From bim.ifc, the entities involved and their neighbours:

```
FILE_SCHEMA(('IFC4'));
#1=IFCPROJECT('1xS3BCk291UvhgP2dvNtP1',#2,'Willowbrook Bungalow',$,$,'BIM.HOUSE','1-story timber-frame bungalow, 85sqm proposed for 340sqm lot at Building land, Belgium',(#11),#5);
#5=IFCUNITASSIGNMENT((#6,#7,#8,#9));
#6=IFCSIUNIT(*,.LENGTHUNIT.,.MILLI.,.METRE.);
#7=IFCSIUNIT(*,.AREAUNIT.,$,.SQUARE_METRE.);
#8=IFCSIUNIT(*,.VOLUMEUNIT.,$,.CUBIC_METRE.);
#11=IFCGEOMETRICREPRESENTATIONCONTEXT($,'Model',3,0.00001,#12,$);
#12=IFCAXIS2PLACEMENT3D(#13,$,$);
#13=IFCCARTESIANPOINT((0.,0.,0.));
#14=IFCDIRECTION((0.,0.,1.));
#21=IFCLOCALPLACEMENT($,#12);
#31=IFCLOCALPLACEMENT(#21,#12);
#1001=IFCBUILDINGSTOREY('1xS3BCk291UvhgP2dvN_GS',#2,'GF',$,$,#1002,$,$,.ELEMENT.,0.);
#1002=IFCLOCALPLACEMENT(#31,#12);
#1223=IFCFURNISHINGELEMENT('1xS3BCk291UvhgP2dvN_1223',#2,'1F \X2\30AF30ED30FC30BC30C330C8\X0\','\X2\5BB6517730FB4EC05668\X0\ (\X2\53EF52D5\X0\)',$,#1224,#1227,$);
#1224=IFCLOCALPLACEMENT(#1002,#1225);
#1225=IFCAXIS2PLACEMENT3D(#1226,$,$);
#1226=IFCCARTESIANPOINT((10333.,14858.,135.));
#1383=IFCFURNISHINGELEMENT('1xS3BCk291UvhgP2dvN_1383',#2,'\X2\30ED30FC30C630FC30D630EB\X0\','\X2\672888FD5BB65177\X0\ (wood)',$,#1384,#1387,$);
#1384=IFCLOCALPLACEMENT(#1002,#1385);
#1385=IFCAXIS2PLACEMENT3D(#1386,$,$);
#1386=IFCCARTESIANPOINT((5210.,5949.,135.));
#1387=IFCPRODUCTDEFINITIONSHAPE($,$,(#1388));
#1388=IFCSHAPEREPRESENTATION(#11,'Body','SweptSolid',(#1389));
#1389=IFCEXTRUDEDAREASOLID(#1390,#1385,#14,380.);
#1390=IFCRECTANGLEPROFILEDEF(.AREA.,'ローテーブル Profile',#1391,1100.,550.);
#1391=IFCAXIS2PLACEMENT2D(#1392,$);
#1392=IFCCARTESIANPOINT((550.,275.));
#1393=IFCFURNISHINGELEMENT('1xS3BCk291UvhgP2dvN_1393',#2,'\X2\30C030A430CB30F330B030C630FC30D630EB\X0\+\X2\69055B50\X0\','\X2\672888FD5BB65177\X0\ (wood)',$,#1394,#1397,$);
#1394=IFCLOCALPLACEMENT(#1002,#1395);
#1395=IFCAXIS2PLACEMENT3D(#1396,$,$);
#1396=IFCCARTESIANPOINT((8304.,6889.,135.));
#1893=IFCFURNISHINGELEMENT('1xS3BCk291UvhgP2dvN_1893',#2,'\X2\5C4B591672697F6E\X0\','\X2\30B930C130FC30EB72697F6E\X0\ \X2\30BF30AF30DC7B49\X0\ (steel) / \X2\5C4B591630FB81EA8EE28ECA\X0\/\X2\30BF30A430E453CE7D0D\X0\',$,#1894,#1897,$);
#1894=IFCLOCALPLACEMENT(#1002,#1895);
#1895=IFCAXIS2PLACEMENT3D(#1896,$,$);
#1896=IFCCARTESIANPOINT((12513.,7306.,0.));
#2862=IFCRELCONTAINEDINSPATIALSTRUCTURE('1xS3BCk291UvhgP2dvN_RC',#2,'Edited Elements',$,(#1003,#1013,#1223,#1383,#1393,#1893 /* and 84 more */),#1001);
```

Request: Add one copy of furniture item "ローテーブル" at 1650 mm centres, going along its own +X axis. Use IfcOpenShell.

```python
import ifcopenshell
import ifcopenshell.api.geometry
import ifcopenshell.api.root
import ifcopenshell.util.element
import ifcopenshell.util.placement
import ifcopenshell.util.unit

model = ifcopenshell.open("bim.ifc")
unit_scale = ifcopenshell.util.unit.calculate_unit_scale(model)


def reuse_history(source, copy):
    """copy_class also copies each property set's owner history, people and application; keep the originals."""
    for rel in copy.IsDefinedBy:
        if rel.is_a("IfcRelDefinesByProperties") and (history := rel.RelatingPropertyDefinition.OwnerHistory):
            rel.RelatingPropertyDefinition.OwnerHistory = source.OwnerHistory
            ifcopenshell.util.element.remove_deep2(model, history)


source = model.by_guid("1xS3BCk291UvhgP2dvN_1383")
base = ifcopenshell.util.placement.get_local_placement(source.ObjectPlacement)
step = base[:3, 0] * 1.65 / unit_scale

for i in range(1, 2):
    copy = ifcopenshell.api.root.copy_class(model, product=source)
    copy.Representation = ifcopenshell.util.element.copy_deep(
        model, source.Representation, exclude=["IfcGeometricRepresentationContext", "IfcRepresentationMap"]
    )
    reuse_history(source, copy)
    matrix = base.copy()
    matrix[:3, 3] += i * step
    print("added at", matrix[:3, 3].round(3) + 0.0)
    ifcopenshell.api.geometry.edit_object_placement(model, product=copy, matrix=matrix, is_si=False)

model.write("bim-out.ifc")
```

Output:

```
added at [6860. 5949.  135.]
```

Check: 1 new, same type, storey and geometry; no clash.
